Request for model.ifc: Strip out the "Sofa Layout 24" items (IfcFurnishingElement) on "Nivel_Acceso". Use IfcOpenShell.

First a look at what the model holds.

```python
import ifcopenshell
import ifcopenshell.util.element

model = ifcopenshell.open("model.ifc")
print(model.schema)
storey = next(s for s in model.by_type("IfcBuildingStorey") if s.Name == "Nivel_Acceso")
furniture = [e for e in ifcopenshell.util.element.get_decomposition(storey) if e.is_a("IfcFurnishingElement")]
seen = {}
for e in furniture:
    element_type = ifcopenshell.util.element.get_type(e)
    name = element_type.Name if element_type not in (None, e) else None
    seen[name] = seen.get(name, 0) + 1
for name, count in sorted(seen.items(), key=str):
    print(count, "x", name)
```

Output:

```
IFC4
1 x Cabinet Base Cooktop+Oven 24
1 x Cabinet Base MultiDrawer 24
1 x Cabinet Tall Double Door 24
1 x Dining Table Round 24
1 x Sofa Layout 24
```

```python
import ifcopenshell
import ifcopenshell.api.root
import ifcopenshell.util.element

model = ifcopenshell.open("model.ifc")

storey = next(s for s in model.by_type("IfcBuildingStorey") if s.Name == "Nivel_Acceso")
furniture = [e for e in ifcopenshell.util.element.get_decomposition(storey) if e.is_a("IfcFurnishingElement")]
targets = [e for e in furniture if (t := ifcopenshell.util.element.get_type(e)) not in (None, e) and t.Name == "Sofa Layout 24"]

for e in targets:
    ifcopenshell.api.root.remove_product(model, product=e)
print(len(targets), "removed")

model.write("model_rev.ifc")
```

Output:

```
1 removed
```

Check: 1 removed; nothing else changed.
